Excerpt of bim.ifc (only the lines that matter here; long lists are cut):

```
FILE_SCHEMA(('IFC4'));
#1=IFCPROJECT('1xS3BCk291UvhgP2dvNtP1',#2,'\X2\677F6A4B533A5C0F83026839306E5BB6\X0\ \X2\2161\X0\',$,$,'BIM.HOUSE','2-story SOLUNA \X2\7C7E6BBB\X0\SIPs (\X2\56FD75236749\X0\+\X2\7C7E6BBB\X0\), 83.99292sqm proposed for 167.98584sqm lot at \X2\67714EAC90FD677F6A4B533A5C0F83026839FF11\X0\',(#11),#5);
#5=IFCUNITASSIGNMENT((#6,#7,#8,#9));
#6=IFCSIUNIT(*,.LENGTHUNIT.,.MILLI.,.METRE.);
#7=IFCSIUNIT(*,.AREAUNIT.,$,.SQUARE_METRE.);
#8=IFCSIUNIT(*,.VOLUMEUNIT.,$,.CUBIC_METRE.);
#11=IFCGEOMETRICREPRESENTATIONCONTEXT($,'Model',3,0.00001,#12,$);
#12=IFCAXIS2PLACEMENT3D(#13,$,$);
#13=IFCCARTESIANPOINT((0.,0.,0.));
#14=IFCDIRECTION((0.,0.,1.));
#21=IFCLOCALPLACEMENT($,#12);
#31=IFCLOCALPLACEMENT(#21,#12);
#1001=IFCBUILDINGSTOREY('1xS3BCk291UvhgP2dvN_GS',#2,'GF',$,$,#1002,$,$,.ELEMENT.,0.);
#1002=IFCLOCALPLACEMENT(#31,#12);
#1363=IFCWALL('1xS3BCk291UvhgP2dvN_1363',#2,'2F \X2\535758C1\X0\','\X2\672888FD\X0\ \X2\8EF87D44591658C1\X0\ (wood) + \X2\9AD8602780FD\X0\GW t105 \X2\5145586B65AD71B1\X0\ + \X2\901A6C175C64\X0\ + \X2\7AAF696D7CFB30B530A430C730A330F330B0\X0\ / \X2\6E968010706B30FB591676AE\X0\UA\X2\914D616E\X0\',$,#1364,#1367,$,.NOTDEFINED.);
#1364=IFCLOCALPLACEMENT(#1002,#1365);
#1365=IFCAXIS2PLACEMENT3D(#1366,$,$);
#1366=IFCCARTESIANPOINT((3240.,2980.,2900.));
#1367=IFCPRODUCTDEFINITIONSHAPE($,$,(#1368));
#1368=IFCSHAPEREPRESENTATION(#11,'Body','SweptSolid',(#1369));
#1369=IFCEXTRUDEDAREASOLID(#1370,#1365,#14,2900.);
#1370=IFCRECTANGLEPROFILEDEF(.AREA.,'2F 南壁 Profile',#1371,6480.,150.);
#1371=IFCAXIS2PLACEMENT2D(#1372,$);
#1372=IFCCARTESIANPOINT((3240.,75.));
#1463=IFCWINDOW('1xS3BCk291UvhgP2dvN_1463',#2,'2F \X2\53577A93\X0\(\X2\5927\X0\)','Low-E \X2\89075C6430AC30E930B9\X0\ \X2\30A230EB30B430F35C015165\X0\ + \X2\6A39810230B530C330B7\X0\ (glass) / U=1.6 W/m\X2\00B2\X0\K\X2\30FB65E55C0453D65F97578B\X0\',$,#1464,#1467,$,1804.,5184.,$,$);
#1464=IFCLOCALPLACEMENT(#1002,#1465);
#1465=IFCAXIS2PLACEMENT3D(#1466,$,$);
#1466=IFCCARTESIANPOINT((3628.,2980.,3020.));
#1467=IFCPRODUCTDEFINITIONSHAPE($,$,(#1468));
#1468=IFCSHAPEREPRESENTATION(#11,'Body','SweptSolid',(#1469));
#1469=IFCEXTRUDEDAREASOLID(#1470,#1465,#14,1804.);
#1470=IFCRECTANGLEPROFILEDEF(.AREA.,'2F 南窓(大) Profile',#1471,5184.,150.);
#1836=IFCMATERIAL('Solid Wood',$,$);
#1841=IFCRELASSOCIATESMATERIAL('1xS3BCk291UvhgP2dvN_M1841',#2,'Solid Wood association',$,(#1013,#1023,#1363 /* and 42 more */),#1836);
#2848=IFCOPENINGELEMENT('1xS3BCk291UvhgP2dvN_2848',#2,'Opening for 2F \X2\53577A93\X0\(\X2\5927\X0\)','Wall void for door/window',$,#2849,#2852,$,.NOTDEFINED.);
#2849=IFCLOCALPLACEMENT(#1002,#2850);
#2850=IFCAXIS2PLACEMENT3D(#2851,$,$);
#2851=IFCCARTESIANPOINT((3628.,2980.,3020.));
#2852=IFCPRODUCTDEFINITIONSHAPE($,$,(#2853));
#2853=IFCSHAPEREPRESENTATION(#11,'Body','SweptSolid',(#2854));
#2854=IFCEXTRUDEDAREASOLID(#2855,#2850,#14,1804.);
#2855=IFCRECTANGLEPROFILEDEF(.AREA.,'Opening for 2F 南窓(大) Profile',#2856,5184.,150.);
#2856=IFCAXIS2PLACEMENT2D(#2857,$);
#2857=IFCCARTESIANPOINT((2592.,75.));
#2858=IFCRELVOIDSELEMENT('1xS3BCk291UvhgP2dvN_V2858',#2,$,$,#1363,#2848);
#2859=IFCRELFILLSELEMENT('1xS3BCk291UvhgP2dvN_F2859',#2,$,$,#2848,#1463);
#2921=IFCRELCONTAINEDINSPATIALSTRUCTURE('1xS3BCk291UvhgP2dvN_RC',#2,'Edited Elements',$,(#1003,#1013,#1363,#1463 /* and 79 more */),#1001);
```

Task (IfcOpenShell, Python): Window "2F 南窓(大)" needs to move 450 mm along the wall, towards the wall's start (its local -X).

```python
import ifcopenshell
import ifcopenshell.api.geometry
import ifcopenshell.util.placement

model = ifcopenshell.open("bim.ifc")

window = model.by_guid("1xS3BCk291UvhgP2dvN_1463")
opening = window.FillsVoids[0].RelatingOpeningElement
wall = opening.VoidsElements[0].RelatingBuildingElement

wall_matrix = ifcopenshell.util.placement.get_local_placement(wall.ObjectPlacement)
shift = wall_matrix[:3, 0] * -450.0
before = ifcopenshell.util.placement.get_local_placement(window.ObjectPlacement)[:3, 3].copy()

# The window is not placed relative to its opening, so move both.
for product in (opening, window):
    matrix = ifcopenshell.util.placement.get_local_placement(product.ObjectPlacement)
    matrix[:3, 3] += shift
    ifcopenshell.api.geometry.edit_object_placement(model, product=product, matrix=matrix, is_si=False)

after = ifcopenshell.util.placement.get_local_placement(window.ObjectPlacement)[:3, 3]
print("window moved by", (after - before).round(3) + 0.0)

model.write("bim_v2.ifc")
```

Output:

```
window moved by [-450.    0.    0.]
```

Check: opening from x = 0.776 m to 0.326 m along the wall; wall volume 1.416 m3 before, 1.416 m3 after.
